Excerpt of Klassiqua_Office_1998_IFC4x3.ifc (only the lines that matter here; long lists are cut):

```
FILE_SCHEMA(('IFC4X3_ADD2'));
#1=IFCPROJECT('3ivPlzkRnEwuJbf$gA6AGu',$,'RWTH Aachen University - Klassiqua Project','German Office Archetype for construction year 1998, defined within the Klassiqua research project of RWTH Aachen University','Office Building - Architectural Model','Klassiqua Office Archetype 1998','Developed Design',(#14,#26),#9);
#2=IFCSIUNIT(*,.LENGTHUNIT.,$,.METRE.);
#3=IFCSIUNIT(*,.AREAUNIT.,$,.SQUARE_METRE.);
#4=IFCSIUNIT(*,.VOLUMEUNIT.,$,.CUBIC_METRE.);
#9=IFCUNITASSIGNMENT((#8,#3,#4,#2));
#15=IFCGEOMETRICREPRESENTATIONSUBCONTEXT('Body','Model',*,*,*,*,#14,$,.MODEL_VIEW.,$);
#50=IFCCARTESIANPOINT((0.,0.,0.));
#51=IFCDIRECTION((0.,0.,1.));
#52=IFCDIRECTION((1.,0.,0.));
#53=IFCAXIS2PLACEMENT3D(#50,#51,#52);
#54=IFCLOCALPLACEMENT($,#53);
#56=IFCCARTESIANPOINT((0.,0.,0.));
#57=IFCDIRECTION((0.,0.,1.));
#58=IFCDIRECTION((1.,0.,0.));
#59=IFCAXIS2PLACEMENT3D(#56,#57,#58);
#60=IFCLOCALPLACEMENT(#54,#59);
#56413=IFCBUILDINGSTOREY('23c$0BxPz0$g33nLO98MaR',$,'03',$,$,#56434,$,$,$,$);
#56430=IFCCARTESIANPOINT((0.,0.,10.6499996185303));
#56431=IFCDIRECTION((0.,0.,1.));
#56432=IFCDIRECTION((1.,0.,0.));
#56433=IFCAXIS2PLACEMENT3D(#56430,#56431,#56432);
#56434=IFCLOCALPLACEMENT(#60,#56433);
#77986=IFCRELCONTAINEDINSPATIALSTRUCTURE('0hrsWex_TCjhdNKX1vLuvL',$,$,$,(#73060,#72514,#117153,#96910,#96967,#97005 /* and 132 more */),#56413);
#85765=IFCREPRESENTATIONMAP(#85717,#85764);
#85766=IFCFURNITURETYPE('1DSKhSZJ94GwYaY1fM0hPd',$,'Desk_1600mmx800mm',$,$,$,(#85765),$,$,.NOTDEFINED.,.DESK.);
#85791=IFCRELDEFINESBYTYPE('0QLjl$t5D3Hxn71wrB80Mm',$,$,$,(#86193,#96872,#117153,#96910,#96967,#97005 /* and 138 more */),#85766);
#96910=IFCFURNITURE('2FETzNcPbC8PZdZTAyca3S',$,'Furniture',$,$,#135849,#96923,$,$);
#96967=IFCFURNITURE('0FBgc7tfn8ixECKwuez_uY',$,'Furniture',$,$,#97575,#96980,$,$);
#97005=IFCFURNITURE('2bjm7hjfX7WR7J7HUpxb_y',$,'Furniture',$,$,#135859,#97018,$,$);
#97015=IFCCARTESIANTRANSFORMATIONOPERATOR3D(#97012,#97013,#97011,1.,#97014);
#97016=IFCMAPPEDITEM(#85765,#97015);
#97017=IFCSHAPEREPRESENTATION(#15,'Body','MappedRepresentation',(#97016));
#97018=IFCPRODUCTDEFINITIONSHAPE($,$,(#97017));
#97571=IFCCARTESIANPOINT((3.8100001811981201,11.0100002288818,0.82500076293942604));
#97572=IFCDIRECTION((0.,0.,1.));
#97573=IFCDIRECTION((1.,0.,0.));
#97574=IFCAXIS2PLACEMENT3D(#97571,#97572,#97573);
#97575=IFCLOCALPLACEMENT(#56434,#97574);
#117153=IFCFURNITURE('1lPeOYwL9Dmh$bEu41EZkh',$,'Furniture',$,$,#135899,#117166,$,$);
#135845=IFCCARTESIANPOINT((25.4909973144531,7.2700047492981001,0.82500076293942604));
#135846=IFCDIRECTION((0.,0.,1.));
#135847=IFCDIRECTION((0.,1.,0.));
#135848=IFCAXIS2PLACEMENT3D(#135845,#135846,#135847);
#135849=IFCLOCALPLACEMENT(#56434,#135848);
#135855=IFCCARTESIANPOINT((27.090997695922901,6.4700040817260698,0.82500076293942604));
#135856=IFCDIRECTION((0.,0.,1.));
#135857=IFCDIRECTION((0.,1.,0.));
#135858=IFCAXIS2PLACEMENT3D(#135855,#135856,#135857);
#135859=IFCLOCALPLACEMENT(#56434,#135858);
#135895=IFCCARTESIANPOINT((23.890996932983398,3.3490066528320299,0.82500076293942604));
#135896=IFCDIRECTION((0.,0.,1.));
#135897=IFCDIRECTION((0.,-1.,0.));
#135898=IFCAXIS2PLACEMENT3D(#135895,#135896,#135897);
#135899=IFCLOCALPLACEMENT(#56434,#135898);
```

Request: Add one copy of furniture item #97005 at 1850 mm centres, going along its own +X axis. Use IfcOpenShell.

```python
import ifcopenshell
import ifcopenshell.api.geometry
import ifcopenshell.api.root
import ifcopenshell.util.element
import ifcopenshell.util.placement
import ifcopenshell.util.unit

model = ifcopenshell.open("Klassiqua_Office_1998_IFC4x3.ifc")
unit_scale = ifcopenshell.util.unit.calculate_unit_scale(model)

source = model.by_guid("2bjm7hjfX7WR7J7HUpxb_y")
base = ifcopenshell.util.placement.get_local_placement(source.ObjectPlacement)
step = base[:3, 0] * 1.85 / unit_scale

for i in range(1, 2):
    copy = ifcopenshell.api.root.copy_class(model, product=source)
    copy.Representation = ifcopenshell.util.element.copy_deep(
        model, source.Representation, exclude=["IfcGeometricRepresentationContext", "IfcRepresentationMap"]
    )
    matrix = base.copy()
    matrix[:3, 3] += i * step
    print("added at", matrix[:3, 3].round(3) + 0.0)
    ifcopenshell.api.geometry.edit_object_placement(model, product=copy, matrix=matrix, is_si=False)

model.write("Klassiqua_Office_1998_IFC4x3_edited.ifc")
```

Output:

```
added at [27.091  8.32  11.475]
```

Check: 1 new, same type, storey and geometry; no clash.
